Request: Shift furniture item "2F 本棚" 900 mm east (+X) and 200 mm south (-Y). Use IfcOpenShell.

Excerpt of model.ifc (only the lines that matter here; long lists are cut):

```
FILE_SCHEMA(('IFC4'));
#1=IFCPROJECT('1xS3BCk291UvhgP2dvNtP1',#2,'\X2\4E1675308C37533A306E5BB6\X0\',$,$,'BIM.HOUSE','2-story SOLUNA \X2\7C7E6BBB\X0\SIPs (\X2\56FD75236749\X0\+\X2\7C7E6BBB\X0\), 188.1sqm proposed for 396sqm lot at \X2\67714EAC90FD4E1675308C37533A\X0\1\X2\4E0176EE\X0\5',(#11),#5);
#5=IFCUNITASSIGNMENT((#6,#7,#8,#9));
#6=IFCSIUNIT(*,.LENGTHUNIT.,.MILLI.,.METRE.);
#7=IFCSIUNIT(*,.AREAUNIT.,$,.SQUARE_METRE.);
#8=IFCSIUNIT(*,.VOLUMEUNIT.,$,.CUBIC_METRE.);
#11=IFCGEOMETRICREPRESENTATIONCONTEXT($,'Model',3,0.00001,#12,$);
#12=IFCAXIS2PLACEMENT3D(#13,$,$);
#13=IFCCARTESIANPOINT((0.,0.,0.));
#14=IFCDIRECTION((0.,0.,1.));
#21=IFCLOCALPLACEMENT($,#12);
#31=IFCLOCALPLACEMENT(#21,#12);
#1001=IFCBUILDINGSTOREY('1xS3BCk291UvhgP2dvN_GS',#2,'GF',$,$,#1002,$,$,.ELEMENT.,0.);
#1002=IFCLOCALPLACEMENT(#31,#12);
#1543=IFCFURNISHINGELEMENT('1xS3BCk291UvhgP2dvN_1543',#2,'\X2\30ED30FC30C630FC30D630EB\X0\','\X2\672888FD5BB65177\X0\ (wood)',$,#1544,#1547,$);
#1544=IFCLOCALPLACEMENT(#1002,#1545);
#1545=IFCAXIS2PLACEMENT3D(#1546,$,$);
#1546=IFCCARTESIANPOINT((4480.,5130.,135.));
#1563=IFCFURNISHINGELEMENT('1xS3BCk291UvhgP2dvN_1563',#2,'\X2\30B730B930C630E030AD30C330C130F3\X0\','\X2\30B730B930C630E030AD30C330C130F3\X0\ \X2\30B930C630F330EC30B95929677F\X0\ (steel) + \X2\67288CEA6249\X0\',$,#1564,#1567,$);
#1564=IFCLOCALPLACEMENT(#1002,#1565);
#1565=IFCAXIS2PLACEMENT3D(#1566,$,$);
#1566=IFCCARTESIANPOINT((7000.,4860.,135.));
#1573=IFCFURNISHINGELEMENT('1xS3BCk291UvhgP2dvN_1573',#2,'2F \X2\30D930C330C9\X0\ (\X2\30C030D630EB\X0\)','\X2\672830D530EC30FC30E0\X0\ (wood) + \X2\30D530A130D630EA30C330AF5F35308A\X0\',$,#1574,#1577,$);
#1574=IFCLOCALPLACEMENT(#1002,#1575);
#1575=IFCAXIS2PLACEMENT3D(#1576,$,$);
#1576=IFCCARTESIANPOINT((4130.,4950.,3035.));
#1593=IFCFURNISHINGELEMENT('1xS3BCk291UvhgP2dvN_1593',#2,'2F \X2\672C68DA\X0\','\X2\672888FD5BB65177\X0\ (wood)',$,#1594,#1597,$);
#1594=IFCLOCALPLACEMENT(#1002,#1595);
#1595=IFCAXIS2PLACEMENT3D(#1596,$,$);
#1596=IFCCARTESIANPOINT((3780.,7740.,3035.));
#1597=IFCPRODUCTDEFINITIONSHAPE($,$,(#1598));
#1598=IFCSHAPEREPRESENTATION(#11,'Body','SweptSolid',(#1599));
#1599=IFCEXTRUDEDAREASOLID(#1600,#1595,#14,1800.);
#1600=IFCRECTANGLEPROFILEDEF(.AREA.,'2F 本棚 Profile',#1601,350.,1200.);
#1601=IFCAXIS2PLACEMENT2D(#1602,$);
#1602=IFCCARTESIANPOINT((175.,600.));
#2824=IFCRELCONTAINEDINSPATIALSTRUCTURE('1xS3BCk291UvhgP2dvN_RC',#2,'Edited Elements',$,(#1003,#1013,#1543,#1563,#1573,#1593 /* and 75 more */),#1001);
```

```python
import ifcopenshell
import ifcopenshell.api.geometry
import ifcopenshell.util.placement

model = ifcopenshell.open("model.ifc")

item = model.by_guid("1xS3BCk291UvhgP2dvN_1593")
matrix = ifcopenshell.util.placement.get_local_placement(item.ObjectPlacement)
matrix[0, 3] += 900.0
matrix[1, 3] -= 200.0
ifcopenshell.api.geometry.edit_object_placement(model, product=item, matrix=matrix, is_si=False)

print(ifcopenshell.util.placement.get_local_placement(item.ObjectPlacement).round(3) + 0.0)

model.write("model_updated.ifc")
```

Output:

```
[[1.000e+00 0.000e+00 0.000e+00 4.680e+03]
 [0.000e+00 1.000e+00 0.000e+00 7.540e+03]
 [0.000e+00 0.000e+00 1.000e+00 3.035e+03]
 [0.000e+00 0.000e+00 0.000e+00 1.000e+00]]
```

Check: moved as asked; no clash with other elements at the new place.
